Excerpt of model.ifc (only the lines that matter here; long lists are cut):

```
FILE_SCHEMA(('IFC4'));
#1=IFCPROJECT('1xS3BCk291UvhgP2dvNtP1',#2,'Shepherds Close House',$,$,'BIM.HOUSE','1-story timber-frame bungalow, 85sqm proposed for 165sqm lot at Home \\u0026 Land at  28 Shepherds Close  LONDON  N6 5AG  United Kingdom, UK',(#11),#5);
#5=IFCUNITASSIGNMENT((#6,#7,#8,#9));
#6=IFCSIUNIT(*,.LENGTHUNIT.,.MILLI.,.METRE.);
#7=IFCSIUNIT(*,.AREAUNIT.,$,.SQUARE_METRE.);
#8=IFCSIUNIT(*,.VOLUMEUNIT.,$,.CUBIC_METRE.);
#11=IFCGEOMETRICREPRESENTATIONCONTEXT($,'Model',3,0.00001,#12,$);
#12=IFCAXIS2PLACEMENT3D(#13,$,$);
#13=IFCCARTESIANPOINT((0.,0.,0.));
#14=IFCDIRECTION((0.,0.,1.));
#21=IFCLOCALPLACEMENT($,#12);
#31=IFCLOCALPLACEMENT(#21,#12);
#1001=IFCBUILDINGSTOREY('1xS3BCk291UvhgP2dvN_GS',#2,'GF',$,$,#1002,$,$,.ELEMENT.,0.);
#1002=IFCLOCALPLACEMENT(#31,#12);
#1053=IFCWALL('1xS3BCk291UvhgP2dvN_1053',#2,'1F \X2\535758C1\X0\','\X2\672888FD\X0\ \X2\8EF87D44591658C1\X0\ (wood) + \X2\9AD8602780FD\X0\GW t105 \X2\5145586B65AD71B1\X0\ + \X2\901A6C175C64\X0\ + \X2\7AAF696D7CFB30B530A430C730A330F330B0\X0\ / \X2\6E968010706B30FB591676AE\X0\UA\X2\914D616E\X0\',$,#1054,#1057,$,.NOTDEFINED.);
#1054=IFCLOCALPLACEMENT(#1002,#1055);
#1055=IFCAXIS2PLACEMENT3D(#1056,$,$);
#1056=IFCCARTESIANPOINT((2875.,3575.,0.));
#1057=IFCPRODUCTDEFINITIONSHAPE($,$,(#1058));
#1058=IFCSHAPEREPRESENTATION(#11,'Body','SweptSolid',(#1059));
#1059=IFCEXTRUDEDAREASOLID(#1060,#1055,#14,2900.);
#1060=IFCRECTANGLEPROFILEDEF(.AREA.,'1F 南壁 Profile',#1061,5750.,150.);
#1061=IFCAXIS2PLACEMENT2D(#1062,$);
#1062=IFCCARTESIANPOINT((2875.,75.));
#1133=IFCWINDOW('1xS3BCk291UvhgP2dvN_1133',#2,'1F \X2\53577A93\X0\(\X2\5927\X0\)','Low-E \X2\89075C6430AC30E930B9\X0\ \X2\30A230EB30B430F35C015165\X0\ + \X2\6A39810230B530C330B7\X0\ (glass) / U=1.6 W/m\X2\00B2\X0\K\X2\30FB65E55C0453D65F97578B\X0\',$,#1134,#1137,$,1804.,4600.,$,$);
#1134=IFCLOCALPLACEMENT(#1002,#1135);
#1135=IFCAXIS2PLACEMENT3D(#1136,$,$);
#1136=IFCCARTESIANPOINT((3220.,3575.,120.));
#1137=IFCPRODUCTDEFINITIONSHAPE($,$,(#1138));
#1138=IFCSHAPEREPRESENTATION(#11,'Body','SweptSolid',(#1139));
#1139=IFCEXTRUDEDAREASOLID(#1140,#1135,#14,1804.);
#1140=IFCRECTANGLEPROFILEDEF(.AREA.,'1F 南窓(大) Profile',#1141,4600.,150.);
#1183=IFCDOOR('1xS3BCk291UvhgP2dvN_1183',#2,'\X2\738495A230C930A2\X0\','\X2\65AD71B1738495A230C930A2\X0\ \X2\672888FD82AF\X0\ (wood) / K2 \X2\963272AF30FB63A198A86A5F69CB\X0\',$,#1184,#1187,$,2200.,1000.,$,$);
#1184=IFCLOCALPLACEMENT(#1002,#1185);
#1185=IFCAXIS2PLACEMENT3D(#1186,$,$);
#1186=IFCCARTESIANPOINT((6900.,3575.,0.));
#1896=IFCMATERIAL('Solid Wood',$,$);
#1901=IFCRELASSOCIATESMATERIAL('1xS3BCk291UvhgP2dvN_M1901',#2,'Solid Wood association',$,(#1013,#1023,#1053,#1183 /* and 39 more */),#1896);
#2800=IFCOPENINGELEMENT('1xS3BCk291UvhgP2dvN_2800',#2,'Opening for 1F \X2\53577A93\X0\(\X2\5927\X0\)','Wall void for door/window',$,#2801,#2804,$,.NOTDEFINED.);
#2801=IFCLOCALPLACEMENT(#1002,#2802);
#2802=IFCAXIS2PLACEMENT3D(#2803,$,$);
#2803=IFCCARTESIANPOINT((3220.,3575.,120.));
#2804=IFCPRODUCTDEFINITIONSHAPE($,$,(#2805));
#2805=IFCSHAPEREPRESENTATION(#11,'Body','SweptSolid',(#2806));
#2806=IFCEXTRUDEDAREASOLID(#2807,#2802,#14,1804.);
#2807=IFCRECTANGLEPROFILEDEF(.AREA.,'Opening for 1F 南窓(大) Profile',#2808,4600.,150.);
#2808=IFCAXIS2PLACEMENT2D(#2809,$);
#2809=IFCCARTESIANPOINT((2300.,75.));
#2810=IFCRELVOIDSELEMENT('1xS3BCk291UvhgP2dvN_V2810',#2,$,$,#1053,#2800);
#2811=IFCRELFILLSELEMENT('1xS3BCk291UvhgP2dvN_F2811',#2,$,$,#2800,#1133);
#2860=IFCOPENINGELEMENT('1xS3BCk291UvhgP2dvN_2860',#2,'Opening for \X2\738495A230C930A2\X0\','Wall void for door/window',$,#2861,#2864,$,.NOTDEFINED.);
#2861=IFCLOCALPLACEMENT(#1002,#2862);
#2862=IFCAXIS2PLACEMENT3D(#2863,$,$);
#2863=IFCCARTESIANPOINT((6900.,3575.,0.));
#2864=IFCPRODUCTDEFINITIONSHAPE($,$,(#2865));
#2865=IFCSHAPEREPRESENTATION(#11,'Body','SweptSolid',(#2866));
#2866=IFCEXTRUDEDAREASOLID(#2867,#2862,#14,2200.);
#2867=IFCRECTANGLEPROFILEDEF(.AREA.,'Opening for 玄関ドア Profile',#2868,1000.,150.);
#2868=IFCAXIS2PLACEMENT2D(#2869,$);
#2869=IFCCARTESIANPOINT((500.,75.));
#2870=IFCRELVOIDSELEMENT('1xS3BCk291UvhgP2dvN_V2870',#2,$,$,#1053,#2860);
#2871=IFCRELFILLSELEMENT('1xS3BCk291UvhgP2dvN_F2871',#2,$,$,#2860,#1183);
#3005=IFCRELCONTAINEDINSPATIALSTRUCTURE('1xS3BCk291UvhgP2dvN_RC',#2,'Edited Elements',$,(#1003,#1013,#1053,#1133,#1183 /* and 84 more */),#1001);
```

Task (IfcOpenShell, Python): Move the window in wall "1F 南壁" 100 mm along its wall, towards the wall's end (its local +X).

```python
import ifcopenshell
import ifcopenshell.api.geometry
import ifcopenshell.util.placement

model = ifcopenshell.open("model.ifc")

window = model.by_id(1133)
opening = window.FillsVoids[0].RelatingOpeningElement
wall = opening.VoidsElements[0].RelatingBuildingElement

wall_matrix = ifcopenshell.util.placement.get_local_placement(wall.ObjectPlacement)
shift = wall_matrix[:3, 0] * 100.0
before = ifcopenshell.util.placement.get_local_placement(window.ObjectPlacement)[:3, 3].copy()

# The window is not placed relative to its opening, so move both.
for product in (opening, window):
    matrix = ifcopenshell.util.placement.get_local_placement(product.ObjectPlacement)
    matrix[:3, 3] += shift
    ifcopenshell.api.geometry.edit_object_placement(model, product=product, matrix=matrix, is_si=False)

after = ifcopenshell.util.placement.get_local_placement(window.ObjectPlacement)[:3, 3]
print("window moved by", (after - before).round(3) + 0.0)

model.write("model_edited.ifc")
```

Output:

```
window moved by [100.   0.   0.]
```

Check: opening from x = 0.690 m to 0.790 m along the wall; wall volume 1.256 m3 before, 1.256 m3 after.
